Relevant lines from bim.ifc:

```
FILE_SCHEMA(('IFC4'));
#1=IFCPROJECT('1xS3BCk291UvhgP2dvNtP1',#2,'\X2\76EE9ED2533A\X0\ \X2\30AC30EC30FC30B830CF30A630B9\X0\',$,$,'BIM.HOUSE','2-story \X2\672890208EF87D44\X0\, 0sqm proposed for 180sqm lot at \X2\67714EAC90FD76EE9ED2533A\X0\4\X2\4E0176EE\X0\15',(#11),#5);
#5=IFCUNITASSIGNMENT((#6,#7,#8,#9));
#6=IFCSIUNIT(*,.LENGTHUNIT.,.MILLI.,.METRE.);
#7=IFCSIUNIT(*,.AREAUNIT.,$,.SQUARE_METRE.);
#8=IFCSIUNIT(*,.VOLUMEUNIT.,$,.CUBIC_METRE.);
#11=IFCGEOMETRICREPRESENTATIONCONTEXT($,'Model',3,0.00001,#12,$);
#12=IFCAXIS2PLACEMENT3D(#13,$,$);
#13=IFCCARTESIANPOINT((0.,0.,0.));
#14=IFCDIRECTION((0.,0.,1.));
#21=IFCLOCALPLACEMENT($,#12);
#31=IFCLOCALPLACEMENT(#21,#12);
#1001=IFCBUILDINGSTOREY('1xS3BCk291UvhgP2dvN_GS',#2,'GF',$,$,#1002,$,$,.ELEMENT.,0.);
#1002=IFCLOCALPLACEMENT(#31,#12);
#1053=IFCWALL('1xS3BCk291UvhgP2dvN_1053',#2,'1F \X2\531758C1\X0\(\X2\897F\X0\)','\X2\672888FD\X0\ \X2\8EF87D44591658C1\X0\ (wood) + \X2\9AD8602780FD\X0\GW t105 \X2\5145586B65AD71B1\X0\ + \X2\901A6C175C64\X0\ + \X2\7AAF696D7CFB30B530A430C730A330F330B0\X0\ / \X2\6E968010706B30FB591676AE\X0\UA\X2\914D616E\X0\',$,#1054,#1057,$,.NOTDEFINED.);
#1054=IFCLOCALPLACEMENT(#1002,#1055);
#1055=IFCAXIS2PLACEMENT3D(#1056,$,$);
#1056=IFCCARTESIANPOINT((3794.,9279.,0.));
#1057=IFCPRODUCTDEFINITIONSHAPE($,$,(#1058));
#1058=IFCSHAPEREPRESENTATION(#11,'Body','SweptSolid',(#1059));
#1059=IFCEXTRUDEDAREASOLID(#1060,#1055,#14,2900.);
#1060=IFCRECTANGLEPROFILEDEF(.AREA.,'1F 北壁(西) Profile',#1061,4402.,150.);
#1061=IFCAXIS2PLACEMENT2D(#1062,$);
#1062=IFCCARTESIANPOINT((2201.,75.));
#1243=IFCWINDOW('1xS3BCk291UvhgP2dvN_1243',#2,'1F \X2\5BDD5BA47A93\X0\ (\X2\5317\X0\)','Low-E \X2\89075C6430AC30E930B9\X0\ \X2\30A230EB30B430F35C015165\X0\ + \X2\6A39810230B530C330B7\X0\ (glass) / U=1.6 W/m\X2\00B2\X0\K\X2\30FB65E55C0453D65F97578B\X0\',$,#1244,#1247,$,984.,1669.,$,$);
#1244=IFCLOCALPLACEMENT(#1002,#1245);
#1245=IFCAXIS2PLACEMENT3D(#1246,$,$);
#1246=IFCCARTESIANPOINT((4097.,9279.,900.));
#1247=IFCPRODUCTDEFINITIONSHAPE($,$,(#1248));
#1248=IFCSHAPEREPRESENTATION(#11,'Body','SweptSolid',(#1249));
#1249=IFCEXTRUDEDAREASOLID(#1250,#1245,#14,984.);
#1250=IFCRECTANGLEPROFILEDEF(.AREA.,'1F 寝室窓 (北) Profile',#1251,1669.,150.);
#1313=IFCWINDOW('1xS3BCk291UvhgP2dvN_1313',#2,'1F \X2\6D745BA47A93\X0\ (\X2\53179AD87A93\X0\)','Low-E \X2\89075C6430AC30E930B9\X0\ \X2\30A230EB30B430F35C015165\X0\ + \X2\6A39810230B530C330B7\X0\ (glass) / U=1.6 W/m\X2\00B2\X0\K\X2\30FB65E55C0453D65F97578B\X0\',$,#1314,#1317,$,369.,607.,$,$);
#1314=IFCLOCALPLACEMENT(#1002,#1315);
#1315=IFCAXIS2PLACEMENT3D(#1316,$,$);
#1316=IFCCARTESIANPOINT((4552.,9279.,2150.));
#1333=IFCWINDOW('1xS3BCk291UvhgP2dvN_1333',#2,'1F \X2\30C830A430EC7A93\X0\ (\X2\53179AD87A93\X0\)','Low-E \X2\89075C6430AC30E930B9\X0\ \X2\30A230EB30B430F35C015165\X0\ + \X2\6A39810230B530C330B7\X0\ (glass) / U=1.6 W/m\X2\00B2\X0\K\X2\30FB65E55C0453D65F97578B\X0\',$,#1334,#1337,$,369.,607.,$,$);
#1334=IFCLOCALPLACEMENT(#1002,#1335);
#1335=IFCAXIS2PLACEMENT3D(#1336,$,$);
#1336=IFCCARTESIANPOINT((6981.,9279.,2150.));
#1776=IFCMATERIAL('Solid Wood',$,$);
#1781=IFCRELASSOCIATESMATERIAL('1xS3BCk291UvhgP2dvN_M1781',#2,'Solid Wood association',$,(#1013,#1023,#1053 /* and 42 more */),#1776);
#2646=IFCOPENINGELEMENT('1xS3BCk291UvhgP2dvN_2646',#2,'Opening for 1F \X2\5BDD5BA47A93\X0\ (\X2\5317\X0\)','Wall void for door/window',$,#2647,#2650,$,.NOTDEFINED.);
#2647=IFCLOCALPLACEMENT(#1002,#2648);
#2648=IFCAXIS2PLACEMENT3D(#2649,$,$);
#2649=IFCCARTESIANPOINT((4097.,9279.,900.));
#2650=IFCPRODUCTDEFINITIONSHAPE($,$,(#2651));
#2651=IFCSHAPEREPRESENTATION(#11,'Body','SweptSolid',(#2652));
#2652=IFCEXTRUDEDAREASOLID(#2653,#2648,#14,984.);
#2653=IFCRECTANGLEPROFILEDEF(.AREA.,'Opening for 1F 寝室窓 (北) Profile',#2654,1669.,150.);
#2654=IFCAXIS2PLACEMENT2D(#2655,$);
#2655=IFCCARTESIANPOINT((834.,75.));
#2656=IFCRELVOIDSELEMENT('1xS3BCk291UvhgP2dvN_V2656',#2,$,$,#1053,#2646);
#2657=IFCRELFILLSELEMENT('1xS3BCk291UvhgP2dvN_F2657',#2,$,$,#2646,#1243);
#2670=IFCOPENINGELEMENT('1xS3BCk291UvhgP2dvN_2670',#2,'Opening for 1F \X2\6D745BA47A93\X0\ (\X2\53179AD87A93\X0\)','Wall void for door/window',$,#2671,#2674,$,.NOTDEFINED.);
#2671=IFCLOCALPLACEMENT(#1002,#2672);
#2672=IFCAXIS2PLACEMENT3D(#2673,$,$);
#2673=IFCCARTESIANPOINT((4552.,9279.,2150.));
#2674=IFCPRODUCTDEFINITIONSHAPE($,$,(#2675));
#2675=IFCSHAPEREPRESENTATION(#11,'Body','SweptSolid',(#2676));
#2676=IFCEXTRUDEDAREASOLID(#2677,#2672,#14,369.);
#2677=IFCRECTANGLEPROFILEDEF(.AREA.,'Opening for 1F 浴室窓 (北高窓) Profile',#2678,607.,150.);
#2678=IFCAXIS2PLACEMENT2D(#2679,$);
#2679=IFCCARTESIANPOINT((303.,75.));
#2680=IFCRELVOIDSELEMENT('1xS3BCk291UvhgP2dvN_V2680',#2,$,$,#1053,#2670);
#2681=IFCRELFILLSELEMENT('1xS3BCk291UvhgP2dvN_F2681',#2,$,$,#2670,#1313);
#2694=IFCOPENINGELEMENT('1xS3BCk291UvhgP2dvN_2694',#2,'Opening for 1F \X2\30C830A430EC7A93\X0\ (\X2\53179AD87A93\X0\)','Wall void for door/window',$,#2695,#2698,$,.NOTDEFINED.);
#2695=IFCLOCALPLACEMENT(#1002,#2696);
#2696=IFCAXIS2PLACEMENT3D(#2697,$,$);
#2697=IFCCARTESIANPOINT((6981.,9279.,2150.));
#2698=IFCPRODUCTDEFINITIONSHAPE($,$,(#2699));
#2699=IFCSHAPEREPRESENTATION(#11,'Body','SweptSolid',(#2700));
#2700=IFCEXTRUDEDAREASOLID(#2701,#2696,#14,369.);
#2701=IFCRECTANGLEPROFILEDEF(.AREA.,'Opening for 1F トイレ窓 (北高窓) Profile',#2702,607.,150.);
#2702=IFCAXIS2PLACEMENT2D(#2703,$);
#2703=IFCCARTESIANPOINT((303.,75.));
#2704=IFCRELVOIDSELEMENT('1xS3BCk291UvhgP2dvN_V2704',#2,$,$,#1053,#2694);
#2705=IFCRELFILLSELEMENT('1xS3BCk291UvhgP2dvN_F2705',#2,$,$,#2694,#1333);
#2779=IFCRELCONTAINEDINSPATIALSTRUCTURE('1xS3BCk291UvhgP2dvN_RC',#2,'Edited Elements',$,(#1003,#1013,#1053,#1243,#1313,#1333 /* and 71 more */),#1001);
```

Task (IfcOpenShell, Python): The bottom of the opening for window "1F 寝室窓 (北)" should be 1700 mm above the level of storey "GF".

```python
import numpy as np
import ifcopenshell
import ifcopenshell.api.geometry
import ifcopenshell.geom
import ifcopenshell.util.element
import ifcopenshell.util.placement
import ifcopenshell.util.shape
import ifcopenshell.util.unit

model = ifcopenshell.open("bim.ifc")
unit_scale = ifcopenshell.util.unit.calculate_unit_scale(model)

window = model.by_guid("1xS3BCk291UvhgP2dvN_1243")
opening = window.FillsVoids[0].RelatingOpeningElement
storey = ifcopenshell.util.element.get_container(window, ifc_class="IfcBuildingStorey")
level = ifcopenshell.util.placement.get_local_placement(storey.ObjectPlacement)[2, 3]

# The opening's origin need not be at the sill, so measure its lowest point.
shape = ifcopenshell.geom.create_shape(ifcopenshell.geom.settings(), opening)
bottom = ifcopenshell.util.shape.get_shape_bottom_elevation(shape, shape.geometry) / unit_scale
dz = level + 1700.0 - bottom

shift = np.array([0.0, 0.0, dz])
# The window is not placed relative to its opening, so move both.
for product in (opening, window):
    matrix = ifcopenshell.util.placement.get_local_placement(product.ObjectPlacement)
    matrix[:3, 3] += shift
    ifcopenshell.api.geometry.edit_object_placement(model, product=product, matrix=matrix, is_si=False)

print(f"moved by {dz * unit_scale:+.3f} m")

model.write("bim_edited.ifc")
```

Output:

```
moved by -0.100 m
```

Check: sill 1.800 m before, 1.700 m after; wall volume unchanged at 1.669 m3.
